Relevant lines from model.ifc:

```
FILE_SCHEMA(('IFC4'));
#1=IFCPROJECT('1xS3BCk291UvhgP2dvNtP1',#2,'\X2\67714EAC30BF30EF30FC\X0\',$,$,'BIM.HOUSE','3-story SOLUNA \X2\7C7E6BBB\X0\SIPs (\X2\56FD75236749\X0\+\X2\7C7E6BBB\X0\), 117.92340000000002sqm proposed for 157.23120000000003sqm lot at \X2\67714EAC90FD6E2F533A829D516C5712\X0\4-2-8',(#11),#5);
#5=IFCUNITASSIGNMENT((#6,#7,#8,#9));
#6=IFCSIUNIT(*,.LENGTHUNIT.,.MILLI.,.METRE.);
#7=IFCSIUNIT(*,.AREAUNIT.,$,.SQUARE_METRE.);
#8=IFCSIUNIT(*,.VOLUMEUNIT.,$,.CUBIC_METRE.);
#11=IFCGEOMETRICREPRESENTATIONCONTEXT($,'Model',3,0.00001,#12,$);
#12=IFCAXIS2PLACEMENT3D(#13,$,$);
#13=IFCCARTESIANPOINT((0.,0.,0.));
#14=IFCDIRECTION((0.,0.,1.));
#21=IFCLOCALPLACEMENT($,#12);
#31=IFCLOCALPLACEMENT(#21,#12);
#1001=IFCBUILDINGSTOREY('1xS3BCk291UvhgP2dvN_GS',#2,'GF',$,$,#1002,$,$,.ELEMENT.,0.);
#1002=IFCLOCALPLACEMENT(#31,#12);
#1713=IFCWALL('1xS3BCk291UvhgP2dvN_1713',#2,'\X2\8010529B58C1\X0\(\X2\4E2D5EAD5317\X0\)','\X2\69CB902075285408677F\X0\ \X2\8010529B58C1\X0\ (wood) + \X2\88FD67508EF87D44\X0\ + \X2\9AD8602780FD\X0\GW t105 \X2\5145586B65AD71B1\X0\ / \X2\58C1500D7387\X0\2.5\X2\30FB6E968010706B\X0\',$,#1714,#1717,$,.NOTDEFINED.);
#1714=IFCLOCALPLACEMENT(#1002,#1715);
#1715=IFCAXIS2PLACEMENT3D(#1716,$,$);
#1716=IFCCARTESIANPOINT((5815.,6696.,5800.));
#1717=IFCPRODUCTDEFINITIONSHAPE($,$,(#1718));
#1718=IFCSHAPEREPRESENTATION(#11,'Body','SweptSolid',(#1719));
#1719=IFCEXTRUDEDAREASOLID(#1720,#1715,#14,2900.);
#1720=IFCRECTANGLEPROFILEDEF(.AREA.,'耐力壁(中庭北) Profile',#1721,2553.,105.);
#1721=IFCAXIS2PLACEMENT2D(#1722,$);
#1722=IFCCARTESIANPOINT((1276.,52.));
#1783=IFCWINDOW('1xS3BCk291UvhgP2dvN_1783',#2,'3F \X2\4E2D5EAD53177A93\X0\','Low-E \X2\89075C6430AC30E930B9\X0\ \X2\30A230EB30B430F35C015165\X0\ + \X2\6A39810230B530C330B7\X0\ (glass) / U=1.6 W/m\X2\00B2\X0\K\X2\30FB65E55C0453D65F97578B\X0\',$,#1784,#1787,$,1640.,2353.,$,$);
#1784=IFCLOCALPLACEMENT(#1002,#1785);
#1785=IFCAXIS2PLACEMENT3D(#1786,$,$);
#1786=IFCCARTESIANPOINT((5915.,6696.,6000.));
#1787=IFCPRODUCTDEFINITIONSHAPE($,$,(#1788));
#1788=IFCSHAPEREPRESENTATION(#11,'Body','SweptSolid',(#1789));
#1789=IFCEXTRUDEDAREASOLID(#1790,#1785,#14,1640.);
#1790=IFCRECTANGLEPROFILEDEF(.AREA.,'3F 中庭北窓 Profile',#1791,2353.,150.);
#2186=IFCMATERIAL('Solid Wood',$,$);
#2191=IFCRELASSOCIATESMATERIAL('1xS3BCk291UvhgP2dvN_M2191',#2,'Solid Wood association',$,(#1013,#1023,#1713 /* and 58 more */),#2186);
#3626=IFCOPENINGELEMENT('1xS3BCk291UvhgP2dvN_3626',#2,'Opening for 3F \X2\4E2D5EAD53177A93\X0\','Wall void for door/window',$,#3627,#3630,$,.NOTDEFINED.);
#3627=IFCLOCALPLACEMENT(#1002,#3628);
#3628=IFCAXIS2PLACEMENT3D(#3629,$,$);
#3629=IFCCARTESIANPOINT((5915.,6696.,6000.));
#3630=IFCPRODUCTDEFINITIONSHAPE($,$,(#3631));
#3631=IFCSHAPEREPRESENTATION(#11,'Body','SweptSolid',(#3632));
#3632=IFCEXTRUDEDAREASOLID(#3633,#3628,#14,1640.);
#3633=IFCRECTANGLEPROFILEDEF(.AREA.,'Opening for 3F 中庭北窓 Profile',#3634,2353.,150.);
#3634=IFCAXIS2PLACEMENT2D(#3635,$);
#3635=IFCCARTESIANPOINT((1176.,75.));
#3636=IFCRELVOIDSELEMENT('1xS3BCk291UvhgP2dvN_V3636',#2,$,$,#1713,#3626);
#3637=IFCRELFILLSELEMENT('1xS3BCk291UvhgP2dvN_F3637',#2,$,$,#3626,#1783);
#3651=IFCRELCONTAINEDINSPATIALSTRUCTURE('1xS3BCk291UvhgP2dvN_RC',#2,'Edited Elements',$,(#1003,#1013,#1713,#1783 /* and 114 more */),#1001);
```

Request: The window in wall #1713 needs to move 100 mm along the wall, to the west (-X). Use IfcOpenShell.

```python
import ifcopenshell
import ifcopenshell.api.geometry
import ifcopenshell.util.placement

model = ifcopenshell.open("model.ifc")

window = model.by_guid("1xS3BCk291UvhgP2dvN_1783")
opening = window.FillsVoids[0].RelatingOpeningElement
wall = opening.VoidsElements[0].RelatingBuildingElement

wall_matrix = ifcopenshell.util.placement.get_local_placement(wall.ObjectPlacement)
shift = wall_matrix[:3, 0] * -100.0
before = ifcopenshell.util.placement.get_local_placement(window.ObjectPlacement)[:3, 3].copy()

# The window is not placed relative to its opening, so move both.
for product in (opening, window):
    matrix = ifcopenshell.util.placement.get_local_placement(product.ObjectPlacement)
    matrix[:3, 3] += shift
    ifcopenshell.api.geometry.edit_object_placement(model, product=product, matrix=matrix, is_si=False)

after = ifcopenshell.util.placement.get_local_placement(window.ObjectPlacement)[:3, 3]
print("window moved by", (after - before).round(3) + 0.0)

model.write("model_rev.ifc")
```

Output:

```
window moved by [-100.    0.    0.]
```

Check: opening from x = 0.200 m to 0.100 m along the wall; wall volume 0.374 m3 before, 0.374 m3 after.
